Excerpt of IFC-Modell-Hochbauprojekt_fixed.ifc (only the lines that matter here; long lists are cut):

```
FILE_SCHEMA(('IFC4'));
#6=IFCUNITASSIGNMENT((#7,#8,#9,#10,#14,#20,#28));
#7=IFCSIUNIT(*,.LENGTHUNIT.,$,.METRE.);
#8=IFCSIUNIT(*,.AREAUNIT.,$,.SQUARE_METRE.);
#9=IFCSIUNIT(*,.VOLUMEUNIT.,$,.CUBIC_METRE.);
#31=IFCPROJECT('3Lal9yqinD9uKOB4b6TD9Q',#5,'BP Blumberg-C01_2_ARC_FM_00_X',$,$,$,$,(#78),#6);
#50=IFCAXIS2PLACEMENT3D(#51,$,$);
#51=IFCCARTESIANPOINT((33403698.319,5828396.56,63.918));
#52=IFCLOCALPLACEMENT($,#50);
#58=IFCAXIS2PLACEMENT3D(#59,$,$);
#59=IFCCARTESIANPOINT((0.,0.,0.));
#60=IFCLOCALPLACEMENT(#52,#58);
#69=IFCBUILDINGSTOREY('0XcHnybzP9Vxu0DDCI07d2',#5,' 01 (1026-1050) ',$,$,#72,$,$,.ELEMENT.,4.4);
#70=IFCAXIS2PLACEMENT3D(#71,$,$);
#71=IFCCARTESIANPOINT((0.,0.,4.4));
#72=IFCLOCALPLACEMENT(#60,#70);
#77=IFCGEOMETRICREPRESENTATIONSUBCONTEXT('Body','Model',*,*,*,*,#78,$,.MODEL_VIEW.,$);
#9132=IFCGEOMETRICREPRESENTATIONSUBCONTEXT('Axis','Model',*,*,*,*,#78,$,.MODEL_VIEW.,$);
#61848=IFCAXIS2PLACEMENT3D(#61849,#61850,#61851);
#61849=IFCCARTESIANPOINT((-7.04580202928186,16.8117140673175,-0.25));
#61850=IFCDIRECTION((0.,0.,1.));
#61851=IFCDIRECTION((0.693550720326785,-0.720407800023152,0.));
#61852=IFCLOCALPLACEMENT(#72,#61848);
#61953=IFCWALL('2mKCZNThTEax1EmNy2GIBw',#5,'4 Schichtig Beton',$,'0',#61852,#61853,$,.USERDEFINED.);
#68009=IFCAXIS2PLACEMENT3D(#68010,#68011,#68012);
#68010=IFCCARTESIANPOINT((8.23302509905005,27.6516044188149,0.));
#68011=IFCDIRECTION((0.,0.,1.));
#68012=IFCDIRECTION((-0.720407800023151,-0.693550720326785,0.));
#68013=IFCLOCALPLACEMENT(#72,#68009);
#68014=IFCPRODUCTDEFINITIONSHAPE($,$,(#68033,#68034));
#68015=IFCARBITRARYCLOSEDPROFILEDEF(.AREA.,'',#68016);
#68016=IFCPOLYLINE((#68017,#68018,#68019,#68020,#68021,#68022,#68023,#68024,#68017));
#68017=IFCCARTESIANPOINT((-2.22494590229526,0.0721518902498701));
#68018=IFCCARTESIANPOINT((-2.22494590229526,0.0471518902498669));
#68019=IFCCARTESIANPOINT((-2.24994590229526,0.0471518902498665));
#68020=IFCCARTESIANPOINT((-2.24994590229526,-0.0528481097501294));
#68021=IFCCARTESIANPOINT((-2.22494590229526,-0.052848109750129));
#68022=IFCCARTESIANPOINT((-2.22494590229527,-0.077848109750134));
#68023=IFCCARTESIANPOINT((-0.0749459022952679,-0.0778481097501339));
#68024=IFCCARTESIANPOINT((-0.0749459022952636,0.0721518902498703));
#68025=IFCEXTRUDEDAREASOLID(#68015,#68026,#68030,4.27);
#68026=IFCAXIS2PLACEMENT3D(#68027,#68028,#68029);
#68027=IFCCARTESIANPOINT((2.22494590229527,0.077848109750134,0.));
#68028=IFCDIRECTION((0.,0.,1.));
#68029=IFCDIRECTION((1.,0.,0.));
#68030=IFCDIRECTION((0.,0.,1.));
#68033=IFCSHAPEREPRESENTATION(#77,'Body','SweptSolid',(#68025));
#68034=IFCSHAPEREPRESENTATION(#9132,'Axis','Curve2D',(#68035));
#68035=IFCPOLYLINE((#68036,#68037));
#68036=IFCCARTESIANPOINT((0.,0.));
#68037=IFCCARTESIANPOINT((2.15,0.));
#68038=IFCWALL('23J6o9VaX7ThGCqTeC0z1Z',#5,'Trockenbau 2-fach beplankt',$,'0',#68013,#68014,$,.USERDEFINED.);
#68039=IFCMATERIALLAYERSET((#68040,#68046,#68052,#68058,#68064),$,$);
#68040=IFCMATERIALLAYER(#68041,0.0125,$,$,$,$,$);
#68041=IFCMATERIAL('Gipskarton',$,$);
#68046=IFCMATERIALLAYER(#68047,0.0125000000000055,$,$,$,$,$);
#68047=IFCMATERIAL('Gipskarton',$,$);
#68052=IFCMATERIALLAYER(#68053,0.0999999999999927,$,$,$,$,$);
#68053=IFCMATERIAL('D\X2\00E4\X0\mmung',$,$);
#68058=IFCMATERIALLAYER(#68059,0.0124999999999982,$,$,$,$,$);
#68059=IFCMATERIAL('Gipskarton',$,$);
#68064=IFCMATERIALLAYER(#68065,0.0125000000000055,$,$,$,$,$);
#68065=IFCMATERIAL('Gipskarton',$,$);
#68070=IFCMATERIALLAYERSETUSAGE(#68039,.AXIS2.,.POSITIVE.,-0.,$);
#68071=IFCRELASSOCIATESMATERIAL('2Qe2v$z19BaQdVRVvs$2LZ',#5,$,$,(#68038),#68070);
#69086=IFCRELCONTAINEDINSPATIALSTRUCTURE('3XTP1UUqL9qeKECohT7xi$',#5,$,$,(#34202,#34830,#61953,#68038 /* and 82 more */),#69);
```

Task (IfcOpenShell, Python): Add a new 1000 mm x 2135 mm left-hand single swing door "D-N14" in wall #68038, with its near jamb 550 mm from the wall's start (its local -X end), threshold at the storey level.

```python
import numpy as np
import ifcopenshell
import ifcopenshell.api.feature
import ifcopenshell.api.geometry
import ifcopenshell.api.root
import ifcopenshell.api.spatial
import ifcopenshell.geom
import ifcopenshell.util.element
import ifcopenshell.util.placement
import ifcopenshell.util.representation
import ifcopenshell.util.shape
import ifcopenshell.util.unit

model = ifcopenshell.open("IFC-Modell-Hochbauprojekt_fixed.ifc")
unit_scale = ifcopenshell.util.unit.calculate_unit_scale(model)
settings = ifcopenshell.geom.settings()


def volume(element):
    """Net volume in cubic metres, openings subtracted."""
    shape = ifcopenshell.geom.create_shape(settings, element)
    return ifcopenshell.util.shape.get_volume(shape.geometry)


wall = model.by_guid("23J6o9VaX7ThGCqTeC0z1Z")
storey = ifcopenshell.util.element.get_container(wall, ifc_class="IfcBuildingStorey")
context = ifcopenshell.util.representation.get_context(model, "Model", "Body", "MODEL_VIEW")
before = volume(wall)

width, height, from_end, sill = 1, 2.135, 0.55, 0.0  # metres

# The wall runs along its own X axis, and the end named is its -X end.
wall_shape = ifcopenshell.geom.create_shape(settings, wall)
x, y, z = ifcopenshell.util.shape.get_vertices(wall_shape.geometry).T
start = x.min() + from_end
face, thickness = float(y.min()), float(y.max() - y.min())
wall_matrix = ifcopenshell.util.placement.get_local_placement(wall.ObjectPlacement)
level = ifcopenshell.util.placement.get_local_placement(storey.ObjectPlacement)[2, 3]


def in_wall(x, y):
    """Placement at x, y metres in the wall's axes, at sill height."""
    matrix = wall_matrix.copy()
    matrix[:, 3] = wall_matrix @ np.array([x / unit_scale, y / unit_scale, 0.0, 1.0])
    matrix[2, 3] = level + sill / unit_scale
    return matrix


# Opening: a box that overshoots both wall faces by 50 mm.
opening = ifcopenshell.api.root.create_entity(model, ifc_class="IfcOpeningElement", predefined_type="OPENING")
box = ifcopenshell.api.geometry.add_wall_representation(
    model, context=context, length=width, height=height, thickness=thickness + 0.1
)
ifcopenshell.api.geometry.assign_representation(model, product=opening, representation=box)
ifcopenshell.api.geometry.edit_object_placement(model, product=opening, matrix=in_wall(start, face - 0.05), is_si=False)
ifcopenshell.api.feature.add_feature(model, feature=opening, element=wall)

door = ifcopenshell.api.root.create_entity(model, ifc_class="IfcDoor", name="D-N14", predefined_type="DOOR")
door.OverallWidth, door.OverallHeight = width / unit_scale, height / unit_scale
door.OperationType = "SINGLE_SWING_LEFT"
body = ifcopenshell.api.geometry.add_door_representation(
    model,
    context=context,
    overall_width=door.OverallWidth,
    overall_height=door.OverallHeight,
    operation_type="SINGLE_SWING_LEFT",
    lining_properties={"LiningDepth": thickness / unit_scale, "ThresholdDepth": thickness / unit_scale},
)
ifcopenshell.api.geometry.assign_representation(model, product=door, representation=body)
ifcopenshell.api.spatial.assign_container(model, products=[door], relating_structure=storey)
ifcopenshell.api.feature.add_filling(model, opening=opening, element=door)

# The lining spans the wall, so the door starts at the wall face.
ifcopenshell.api.geometry.edit_object_placement(model, product=door, matrix=in_wall(start, face), is_si=False)

after = volume(wall)

print(f"wall volume {before:.3f} -> {after:.3f} m3")

model.write("IFC-Modell-Hochbauprojekt_fixed_rev.ifc")
```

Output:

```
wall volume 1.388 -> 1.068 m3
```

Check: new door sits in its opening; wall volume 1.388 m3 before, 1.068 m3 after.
